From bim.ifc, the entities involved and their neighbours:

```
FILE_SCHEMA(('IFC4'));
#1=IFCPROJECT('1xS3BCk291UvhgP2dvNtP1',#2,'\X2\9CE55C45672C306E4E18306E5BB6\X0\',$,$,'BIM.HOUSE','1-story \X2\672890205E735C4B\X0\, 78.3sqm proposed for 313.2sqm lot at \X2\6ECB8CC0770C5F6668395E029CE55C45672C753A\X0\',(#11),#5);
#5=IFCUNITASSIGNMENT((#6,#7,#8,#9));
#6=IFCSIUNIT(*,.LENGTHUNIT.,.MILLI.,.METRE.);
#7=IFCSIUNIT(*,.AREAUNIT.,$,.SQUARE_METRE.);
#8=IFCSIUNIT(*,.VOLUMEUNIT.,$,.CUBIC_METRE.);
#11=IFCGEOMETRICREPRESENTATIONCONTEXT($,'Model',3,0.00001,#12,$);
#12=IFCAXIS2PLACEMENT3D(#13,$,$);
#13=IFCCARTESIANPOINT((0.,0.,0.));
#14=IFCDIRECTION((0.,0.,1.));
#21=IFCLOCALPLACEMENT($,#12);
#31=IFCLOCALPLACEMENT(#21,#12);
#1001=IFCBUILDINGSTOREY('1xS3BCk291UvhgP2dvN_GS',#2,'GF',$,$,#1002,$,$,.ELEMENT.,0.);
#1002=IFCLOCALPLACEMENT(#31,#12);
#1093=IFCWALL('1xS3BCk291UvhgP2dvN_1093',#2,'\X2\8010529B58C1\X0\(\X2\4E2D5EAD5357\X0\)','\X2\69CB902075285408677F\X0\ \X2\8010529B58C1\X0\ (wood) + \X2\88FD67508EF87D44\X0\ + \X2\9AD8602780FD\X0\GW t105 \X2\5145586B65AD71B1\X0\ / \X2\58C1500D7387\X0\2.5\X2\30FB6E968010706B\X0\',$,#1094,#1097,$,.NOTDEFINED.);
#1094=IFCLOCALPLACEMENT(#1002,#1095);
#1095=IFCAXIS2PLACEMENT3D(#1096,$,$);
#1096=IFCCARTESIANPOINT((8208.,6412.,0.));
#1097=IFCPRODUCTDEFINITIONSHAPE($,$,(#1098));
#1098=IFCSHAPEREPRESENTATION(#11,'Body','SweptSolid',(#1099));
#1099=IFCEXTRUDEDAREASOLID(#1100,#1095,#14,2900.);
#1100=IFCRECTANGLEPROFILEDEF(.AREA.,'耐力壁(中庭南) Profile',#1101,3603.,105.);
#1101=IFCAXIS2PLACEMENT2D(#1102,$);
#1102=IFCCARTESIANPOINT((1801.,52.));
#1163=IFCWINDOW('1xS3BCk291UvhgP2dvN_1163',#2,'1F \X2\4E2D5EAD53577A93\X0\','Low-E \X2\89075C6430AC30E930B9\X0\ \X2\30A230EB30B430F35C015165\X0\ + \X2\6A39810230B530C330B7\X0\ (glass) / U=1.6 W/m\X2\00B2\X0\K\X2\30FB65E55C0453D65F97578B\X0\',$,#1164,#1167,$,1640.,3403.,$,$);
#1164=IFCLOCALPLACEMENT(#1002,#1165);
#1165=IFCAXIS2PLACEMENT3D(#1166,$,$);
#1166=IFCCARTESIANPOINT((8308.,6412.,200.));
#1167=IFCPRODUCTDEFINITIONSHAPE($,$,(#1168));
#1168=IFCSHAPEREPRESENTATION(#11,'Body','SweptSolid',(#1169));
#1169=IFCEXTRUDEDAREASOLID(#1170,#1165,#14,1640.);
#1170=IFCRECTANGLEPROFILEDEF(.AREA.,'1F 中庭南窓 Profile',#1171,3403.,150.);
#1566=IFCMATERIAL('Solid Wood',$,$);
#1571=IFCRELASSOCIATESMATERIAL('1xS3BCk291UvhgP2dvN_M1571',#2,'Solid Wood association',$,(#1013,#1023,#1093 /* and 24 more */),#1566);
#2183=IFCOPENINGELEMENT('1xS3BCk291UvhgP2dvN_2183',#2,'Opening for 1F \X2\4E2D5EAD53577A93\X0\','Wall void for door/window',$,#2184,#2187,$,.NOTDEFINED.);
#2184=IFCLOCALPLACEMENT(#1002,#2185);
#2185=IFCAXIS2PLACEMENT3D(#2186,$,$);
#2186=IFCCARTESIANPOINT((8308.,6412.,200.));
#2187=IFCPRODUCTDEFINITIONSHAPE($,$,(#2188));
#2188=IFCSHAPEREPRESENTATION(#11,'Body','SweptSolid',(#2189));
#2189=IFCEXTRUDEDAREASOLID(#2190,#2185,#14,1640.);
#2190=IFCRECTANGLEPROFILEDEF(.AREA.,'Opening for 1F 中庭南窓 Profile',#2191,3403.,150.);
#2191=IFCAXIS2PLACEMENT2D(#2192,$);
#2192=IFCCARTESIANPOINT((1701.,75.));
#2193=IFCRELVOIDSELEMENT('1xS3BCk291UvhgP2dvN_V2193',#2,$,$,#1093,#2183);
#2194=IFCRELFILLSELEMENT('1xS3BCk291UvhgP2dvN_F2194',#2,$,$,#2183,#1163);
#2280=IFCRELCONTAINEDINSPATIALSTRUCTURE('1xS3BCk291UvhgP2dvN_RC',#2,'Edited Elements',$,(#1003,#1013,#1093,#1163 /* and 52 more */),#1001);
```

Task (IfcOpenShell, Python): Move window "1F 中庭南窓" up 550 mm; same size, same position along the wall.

```python
import numpy as np
import ifcopenshell
import ifcopenshell.api.geometry
import ifcopenshell.util.placement
import ifcopenshell.util.unit

model = ifcopenshell.open("bim.ifc")
unit_scale = ifcopenshell.util.unit.calculate_unit_scale(model)

window = model.by_guid("1xS3BCk291UvhgP2dvN_1163")
opening = window.FillsVoids[0].RelatingOpeningElement
dz = 0.55 / unit_scale

shift = np.array([0.0, 0.0, dz])
# The window is not placed relative to its opening, so move both.
for product in (opening, window):
    matrix = ifcopenshell.util.placement.get_local_placement(product.ObjectPlacement)
    matrix[:3, 3] += shift
    ifcopenshell.api.geometry.edit_object_placement(model, product=product, matrix=matrix, is_si=False)

print(f"moved by {dz * unit_scale:+.3f} m")

model.write("bim_rev.ifc")
```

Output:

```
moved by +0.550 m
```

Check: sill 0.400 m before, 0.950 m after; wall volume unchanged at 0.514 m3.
